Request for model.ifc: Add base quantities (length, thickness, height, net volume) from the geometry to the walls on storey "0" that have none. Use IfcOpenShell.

First a look at what the model holds.

```python
import ifcopenshell
import ifcopenshell.util.element
import ifcopenshell.util.unit

model = ifcopenshell.open("model.ifc")
print(model.schema)
for unit_type in ("LENGTHUNIT", "AREAUNIT", "VOLUMEUNIT"):
    print(unit_type, ifcopenshell.util.unit.calculate_unit_scale(model, unit_type))
storey = next(s for s in model.by_type("IfcBuildingStorey") if s.Name == "0")
walls = [e for e in ifcopenshell.util.element.get_decomposition(storey) if e.is_a("IfcWall")]
for e in sorted(walls, key=lambda e: e.id()):
    print(e.id(), e.is_a(), e.Name, list(ifcopenshell.util.element.get_psets(e, qtos_only=True)), sep=" | ")
```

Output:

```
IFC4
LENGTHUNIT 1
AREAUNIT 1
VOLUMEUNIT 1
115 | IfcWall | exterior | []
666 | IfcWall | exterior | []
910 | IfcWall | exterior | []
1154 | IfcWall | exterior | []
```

```python
import ifcopenshell
import ifcopenshell.api.pset
import ifcopenshell.geom
import ifcopenshell.util.element
import ifcopenshell.util.shape
import ifcopenshell.util.unit

model = ifcopenshell.open("model.ifc")
unit_scale = ifcopenshell.util.unit.calculate_unit_scale(model)
volume_scale = ifcopenshell.util.unit.calculate_unit_scale(model, "VOLUMEUNIT")
settings = ifcopenshell.geom.settings()

storey = next(s for s in model.by_type("IfcBuildingStorey") if s.Name == "0")
walls = [e for e in ifcopenshell.util.element.get_decomposition(storey) if e.is_a("IfcWall")]

for e in sorted(walls, key=lambda e: e.id()):
    if ifcopenshell.util.element.get_psets(e, qtos_only=True, should_inherit=False):
        continue
    # Geometry comes back in metres, in the element's own axes.
    shape = ifcopenshell.geom.create_shape(settings, e)
    values = {
        "Length": ifcopenshell.util.shape.get_x(shape.geometry) / unit_scale,
        "Width": ifcopenshell.util.shape.get_y(shape.geometry) / unit_scale,
        "Height": ifcopenshell.util.shape.get_z(shape.geometry) / unit_scale,
        "NetVolume": ifcopenshell.util.shape.get_volume(shape.geometry) / volume_scale,
    }
    qto = ifcopenshell.api.pset.add_qto(model, product=e, name="Qto_WallBaseQuantities")
    ifcopenshell.api.pset.edit_qto(model, qto=qto, properties=values)
    print(e.id(), {k: round(v, 3) for k, v in values.items()})

model.write("model_v2.ifc")
```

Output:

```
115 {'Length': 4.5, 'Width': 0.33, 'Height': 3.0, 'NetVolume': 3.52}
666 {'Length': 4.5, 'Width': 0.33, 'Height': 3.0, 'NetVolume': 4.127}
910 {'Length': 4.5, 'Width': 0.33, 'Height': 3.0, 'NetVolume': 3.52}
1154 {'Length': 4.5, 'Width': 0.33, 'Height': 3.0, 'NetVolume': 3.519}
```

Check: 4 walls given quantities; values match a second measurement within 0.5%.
